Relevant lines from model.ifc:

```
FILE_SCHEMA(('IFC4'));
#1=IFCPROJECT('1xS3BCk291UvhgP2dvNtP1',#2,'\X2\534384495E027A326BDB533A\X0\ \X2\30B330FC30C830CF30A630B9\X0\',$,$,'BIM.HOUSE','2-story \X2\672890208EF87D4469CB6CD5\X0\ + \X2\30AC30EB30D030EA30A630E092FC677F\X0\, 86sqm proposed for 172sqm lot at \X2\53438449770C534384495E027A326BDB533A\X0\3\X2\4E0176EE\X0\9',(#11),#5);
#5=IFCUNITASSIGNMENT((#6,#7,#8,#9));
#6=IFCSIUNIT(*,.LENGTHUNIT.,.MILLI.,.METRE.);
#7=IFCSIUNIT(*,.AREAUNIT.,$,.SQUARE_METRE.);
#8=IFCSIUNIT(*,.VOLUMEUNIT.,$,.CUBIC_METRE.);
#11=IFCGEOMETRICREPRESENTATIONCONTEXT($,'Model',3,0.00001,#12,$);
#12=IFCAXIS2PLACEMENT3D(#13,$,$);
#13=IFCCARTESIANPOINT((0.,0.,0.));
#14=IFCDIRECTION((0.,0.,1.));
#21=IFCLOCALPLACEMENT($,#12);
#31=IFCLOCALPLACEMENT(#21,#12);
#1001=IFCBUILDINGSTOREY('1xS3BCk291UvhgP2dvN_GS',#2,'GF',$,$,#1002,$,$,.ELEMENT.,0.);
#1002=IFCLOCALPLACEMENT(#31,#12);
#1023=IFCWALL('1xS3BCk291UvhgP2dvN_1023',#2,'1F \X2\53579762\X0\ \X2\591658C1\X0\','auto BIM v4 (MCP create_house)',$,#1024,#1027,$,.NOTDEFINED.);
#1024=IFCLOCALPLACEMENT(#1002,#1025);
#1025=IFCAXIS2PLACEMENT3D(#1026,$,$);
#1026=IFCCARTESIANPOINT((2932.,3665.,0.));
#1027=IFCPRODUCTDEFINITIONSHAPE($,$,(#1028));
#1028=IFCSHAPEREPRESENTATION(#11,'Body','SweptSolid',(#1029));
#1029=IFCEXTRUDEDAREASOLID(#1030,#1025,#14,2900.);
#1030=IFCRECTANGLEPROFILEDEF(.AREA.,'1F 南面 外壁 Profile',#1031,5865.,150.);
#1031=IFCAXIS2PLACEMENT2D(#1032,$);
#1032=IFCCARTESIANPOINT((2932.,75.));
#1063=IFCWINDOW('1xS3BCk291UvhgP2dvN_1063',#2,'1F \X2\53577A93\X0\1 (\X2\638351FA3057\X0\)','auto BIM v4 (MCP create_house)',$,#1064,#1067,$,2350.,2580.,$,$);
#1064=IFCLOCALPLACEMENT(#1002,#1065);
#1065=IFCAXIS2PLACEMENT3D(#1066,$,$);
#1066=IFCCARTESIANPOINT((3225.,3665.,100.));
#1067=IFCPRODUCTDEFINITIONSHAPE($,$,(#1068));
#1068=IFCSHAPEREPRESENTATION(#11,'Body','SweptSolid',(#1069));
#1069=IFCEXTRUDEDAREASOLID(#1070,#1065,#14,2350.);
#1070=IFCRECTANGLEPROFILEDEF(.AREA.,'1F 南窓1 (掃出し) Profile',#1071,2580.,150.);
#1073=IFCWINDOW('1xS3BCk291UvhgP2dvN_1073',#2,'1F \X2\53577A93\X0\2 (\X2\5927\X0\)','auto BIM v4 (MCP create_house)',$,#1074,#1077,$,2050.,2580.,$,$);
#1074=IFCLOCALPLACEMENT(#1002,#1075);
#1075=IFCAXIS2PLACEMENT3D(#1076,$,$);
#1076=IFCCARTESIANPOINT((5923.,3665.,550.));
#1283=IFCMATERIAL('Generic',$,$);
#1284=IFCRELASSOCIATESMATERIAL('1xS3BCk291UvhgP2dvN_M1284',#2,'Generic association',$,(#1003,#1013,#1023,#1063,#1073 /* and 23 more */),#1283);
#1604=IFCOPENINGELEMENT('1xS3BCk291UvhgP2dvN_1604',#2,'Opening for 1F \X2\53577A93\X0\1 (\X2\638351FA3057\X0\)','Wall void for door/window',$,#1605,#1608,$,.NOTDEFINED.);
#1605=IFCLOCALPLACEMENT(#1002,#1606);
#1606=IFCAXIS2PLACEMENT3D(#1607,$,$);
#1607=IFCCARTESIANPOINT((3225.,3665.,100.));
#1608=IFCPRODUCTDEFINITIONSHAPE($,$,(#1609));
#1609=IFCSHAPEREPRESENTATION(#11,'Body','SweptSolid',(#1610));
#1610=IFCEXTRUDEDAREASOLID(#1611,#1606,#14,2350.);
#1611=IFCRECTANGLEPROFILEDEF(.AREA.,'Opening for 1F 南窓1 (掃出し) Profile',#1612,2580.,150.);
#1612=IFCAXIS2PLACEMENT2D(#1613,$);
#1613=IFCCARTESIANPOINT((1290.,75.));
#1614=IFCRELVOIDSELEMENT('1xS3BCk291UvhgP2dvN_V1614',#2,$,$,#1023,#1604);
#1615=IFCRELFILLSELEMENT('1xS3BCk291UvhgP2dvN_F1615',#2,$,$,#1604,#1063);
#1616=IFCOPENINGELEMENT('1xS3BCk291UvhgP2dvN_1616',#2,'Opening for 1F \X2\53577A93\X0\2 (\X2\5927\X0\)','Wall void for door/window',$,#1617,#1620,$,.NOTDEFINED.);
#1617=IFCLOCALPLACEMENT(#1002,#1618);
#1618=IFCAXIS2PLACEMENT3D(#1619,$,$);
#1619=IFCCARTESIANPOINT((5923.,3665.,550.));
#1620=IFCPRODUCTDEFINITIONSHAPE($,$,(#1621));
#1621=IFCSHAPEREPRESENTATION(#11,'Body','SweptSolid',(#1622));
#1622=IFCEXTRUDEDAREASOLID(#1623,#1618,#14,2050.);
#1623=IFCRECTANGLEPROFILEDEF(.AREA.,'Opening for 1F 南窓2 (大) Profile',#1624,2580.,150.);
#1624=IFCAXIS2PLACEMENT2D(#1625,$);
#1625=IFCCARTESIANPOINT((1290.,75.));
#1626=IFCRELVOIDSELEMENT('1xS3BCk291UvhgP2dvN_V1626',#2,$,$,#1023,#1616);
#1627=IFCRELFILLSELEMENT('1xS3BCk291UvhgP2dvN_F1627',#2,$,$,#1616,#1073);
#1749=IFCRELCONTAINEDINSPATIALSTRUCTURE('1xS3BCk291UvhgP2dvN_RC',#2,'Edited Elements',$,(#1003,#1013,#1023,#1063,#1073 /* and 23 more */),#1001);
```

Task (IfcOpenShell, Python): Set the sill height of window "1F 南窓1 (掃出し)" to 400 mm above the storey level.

```python
import numpy as np
import ifcopenshell
import ifcopenshell.api.geometry
import ifcopenshell.geom
import ifcopenshell.util.element
import ifcopenshell.util.placement
import ifcopenshell.util.shape
import ifcopenshell.util.unit

model = ifcopenshell.open("model.ifc")
unit_scale = ifcopenshell.util.unit.calculate_unit_scale(model)

window = model.by_guid("1xS3BCk291UvhgP2dvN_1063")
opening = window.FillsVoids[0].RelatingOpeningElement
storey = ifcopenshell.util.element.get_container(window, ifc_class="IfcBuildingStorey")
level = ifcopenshell.util.placement.get_local_placement(storey.ObjectPlacement)[2, 3]

# The opening's origin need not be at the sill, so measure its lowest point.
shape = ifcopenshell.geom.create_shape(ifcopenshell.geom.settings(), opening)
bottom = ifcopenshell.util.shape.get_shape_bottom_elevation(shape, shape.geometry) / unit_scale
dz = level + 0.4 / unit_scale - bottom

shift = np.array([0.0, 0.0, dz])
# The window is not placed relative to its opening, so move both.
for product in (opening, window):
    matrix = ifcopenshell.util.placement.get_local_placement(product.ObjectPlacement)
    matrix[:3, 3] += shift
    ifcopenshell.api.geometry.edit_object_placement(model, product=product, matrix=matrix, is_si=False)

print(f"moved by {dz * unit_scale:+.3f} m")

model.write("model_updated.ifc")
```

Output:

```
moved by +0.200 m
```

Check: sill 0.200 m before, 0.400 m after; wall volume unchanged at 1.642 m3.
